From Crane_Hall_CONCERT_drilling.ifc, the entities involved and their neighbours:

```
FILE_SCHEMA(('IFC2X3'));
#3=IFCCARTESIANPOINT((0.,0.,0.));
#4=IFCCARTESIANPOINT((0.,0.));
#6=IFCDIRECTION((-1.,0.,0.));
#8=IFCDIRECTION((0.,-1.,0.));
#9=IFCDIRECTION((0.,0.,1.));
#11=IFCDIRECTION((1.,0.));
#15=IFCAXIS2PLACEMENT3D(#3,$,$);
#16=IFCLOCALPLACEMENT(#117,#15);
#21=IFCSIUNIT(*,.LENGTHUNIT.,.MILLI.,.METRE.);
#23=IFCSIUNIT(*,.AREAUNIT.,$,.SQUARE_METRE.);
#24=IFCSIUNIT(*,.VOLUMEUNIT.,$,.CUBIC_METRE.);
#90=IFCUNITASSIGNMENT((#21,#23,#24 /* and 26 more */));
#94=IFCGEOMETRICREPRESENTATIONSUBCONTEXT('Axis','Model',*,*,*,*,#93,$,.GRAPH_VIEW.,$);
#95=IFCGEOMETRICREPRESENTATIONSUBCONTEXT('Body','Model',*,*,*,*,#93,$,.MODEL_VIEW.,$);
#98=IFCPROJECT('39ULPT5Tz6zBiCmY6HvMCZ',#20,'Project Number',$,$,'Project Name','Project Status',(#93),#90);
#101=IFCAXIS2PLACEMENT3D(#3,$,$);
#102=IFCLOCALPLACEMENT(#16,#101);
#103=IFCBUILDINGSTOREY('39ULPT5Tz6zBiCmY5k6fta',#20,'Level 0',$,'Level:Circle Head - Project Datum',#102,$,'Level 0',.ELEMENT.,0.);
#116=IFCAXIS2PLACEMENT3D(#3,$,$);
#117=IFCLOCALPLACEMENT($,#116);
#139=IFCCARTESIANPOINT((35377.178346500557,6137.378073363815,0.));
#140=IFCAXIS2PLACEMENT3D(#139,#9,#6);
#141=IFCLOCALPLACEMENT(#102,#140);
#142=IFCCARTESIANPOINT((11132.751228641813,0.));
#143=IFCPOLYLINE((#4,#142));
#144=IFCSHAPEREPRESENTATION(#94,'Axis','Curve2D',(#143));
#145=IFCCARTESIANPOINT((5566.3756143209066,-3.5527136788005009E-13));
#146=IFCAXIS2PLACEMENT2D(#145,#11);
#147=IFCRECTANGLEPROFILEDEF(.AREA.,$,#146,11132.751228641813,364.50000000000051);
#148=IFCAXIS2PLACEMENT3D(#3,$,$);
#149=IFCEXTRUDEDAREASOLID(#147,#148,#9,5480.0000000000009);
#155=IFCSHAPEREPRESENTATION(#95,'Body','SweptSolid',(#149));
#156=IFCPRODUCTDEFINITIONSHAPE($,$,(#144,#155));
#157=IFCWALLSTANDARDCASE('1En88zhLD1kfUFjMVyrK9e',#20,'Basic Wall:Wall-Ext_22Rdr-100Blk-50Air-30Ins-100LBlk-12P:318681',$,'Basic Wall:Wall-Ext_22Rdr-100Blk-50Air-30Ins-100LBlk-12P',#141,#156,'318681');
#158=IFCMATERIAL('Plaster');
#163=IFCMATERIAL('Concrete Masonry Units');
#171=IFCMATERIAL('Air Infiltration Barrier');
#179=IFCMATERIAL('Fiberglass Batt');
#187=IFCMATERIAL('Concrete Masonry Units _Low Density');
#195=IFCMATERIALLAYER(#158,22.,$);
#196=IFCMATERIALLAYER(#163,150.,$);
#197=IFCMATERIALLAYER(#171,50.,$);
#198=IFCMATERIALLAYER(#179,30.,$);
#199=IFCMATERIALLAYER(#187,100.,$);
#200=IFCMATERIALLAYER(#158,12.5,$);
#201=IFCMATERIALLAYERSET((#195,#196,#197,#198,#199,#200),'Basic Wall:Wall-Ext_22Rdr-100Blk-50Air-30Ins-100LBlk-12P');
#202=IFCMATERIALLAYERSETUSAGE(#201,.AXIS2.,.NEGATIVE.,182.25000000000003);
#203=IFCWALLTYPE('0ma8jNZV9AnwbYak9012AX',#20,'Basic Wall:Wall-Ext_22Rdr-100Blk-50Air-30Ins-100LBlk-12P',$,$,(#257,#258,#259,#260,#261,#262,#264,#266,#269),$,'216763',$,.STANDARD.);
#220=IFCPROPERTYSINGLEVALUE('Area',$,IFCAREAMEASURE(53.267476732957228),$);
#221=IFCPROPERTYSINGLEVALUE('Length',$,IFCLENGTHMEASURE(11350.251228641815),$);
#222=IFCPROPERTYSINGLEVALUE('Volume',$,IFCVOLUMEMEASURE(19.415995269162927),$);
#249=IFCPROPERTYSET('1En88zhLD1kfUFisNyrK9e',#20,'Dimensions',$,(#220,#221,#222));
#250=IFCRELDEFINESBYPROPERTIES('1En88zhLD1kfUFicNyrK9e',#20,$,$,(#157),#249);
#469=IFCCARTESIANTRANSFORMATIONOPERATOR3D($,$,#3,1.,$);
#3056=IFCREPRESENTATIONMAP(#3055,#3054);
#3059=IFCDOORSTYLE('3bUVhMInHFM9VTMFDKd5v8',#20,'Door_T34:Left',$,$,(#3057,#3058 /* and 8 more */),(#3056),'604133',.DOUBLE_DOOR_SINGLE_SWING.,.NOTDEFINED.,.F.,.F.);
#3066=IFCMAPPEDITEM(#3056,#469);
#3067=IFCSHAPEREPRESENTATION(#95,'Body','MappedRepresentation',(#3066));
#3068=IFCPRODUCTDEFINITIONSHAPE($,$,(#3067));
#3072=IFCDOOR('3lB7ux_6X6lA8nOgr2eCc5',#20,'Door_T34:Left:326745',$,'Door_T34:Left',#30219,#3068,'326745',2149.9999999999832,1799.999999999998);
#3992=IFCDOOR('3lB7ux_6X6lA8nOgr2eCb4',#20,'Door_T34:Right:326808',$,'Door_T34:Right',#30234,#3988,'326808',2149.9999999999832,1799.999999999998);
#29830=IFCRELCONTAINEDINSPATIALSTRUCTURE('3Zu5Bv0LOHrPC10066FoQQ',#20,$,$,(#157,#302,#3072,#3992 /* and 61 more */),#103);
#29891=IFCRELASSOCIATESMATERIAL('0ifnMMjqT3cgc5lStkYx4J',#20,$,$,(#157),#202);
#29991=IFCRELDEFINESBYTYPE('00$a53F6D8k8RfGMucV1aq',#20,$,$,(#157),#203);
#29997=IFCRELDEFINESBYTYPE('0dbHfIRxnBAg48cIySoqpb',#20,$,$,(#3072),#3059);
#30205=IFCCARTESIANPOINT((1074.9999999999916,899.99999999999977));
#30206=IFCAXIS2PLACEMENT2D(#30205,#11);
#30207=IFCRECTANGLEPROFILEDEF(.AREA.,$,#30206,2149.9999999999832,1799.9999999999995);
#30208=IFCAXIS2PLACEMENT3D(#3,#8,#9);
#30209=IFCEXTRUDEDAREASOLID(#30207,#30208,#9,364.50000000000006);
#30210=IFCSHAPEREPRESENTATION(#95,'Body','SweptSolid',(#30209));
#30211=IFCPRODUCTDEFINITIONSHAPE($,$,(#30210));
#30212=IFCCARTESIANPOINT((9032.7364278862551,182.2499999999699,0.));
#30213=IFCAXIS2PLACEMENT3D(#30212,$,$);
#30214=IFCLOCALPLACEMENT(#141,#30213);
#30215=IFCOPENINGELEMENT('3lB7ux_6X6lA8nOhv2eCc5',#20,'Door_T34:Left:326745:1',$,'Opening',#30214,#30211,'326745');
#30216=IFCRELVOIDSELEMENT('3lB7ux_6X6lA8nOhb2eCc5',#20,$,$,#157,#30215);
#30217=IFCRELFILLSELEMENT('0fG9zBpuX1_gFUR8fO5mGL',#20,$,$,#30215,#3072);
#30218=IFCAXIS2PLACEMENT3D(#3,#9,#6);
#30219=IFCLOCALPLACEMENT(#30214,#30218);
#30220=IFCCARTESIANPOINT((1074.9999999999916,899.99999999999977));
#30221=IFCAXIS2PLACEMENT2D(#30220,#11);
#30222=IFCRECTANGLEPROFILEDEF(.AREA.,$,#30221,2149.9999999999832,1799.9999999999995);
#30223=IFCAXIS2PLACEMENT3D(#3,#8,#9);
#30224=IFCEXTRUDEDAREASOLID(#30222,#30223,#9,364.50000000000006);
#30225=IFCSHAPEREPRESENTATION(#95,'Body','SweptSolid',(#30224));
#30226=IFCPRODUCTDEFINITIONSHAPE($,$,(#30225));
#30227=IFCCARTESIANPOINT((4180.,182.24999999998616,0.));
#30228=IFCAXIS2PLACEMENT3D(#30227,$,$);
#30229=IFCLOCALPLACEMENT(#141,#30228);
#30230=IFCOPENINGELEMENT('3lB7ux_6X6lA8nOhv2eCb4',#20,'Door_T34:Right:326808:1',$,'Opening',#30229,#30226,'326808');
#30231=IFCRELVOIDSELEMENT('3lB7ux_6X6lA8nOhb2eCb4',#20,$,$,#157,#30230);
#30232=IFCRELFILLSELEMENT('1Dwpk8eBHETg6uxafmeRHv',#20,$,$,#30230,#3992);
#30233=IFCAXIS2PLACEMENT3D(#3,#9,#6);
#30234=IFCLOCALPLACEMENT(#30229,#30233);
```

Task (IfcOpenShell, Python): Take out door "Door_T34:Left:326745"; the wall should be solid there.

```python
import ifcopenshell
import ifcopenshell.api.feature
import ifcopenshell.api.pset
import ifcopenshell.api.root
import ifcopenshell.geom
import ifcopenshell.util.element
import ifcopenshell.util.shape
import ifcopenshell.util.unit

model = ifcopenshell.open("Crane_Hall_CONCERT_drilling.ifc")
area_scale = ifcopenshell.util.unit.calculate_unit_scale(model, "AREAUNIT")
volume_scale = ifcopenshell.util.unit.calculate_unit_scale(model, "VOLUMEUNIT")
settings = ifcopenshell.geom.settings()


def volume(element):
    """Net volume in cubic metres, openings subtracted."""
    shape = ifcopenshell.geom.create_shape(settings, element)
    return ifcopenshell.util.shape.get_volume(shape.geometry)


door = model.by_guid("3lB7ux_6X6lA8nOgr2eCc5")
opening = door.FillsVoids[0].RelatingOpeningElement
wall = opening.VoidsElements[0].RelatingBuildingElement
before = volume(wall)

ifcopenshell.api.root.remove_product(model, product=door)
ifcopenshell.api.feature.remove_feature(model, feature=opening)

after = volume(wall)
thickness = 0.3645  # wall thickness in metres

# Update the wall's stored quantities.
pset = model.by_id(ifcopenshell.util.element.get_pset(wall, "Dimensions", should_inherit=False)["id"])
ifcopenshell.api.pset.edit_pset(model, pset=pset, properties={
    "Area": model.create_entity("IfcAreaMeasure", after / thickness / area_scale),
    "Volume": model.create_entity("IfcVolumeMeasure", after / volume_scale),
})

print(f"wall volume {before:.3f} -> {after:.3f} m3")

model.write("Crane_Hall_CONCERT_drilling-out.ifc")
```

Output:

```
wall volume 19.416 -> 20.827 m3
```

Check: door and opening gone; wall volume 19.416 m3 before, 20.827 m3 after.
